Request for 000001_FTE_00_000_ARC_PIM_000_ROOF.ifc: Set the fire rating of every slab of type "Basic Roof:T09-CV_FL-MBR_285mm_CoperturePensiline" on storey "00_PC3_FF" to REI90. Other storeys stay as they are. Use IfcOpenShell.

First a look at what the model holds.

```python
import ifcopenshell
import ifcopenshell.util.element

model = ifcopenshell.open("000001_FTE_00_000_ARC_PIM_000_ROOF.ifc")
print(model.schema)
storey = next(s for s in model.by_type("IfcBuildingStorey") if s.Name == "00_PC3_FF")
slabs = [e for e in ifcopenshell.util.element.get_decomposition(storey) if e.is_a("IfcSlab")]
seen = {}
for e in slabs:
    element_type = ifcopenshell.util.element.get_type(e)
    key = (element_type.Name if element_type != e and element_type else None, ifcopenshell.util.element.get_pset(e, "Pset_SlabCommon", "FireRating"))
    seen[key] = seen.get(key, 0) + 1
for (name, value), count in sorted(seen.items(), key=str):
    print(count, "x", name, "|", value)
```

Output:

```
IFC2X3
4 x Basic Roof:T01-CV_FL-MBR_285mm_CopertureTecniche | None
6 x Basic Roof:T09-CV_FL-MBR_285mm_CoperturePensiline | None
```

```python
import ifcopenshell
import ifcopenshell.api.pset
import ifcopenshell.util.element

model = ifcopenshell.open("000001_FTE_00_000_ARC_PIM_000_ROOF.ifc")

storey = next(s for s in model.by_type("IfcBuildingStorey") if s.Name == "00_PC3_FF")
slabs = [e for e in ifcopenshell.util.element.get_decomposition(storey) if e.is_a("IfcSlab")]

count = 0
for e in slabs:
    element_type = ifcopenshell.util.element.get_type(e)
    if element_type in (None, e) or element_type.Name != "Basic Roof:T09-CV_FL-MBR_285mm_CoperturePensiline":
        continue
    # add_pset returns the element's existing set when there is one.
    pset = ifcopenshell.api.pset.add_pset(model, product=e, name="Pset_SlabCommon")
    ifcopenshell.api.pset.edit_pset(model, pset=pset, properties={"FireRating": "REI90"})
    count += 1

print(count, "slabs updated")

model.write("000001_FTE_00_000_ARC_PIM_000_ROOF_updated.ifc")
```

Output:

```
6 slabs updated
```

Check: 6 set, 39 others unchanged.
